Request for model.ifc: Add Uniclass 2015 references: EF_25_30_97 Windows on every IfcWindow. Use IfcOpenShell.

First a look at what the model holds.

```python
import ifcopenshell

model = ifcopenshell.open("model.ifc")
print(model.schema)
print("classifications:", [c.Name for c in model.by_type("IfcClassification")])
for ifc_class in ("IfcDoor", "IfcRoof", "IfcStair", "IfcWall", "IfcWindow"):
    print(ifc_class, len(model.by_type(ifc_class)))
```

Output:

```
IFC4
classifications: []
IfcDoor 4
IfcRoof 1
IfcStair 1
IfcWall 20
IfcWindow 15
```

```python
import ifcopenshell
import ifcopenshell.api.classification

model = ifcopenshell.open("model.ifc")

system = ifcopenshell.api.classification.add_classification(model, classification="Uniclass 2015")

codes = {
    "IfcWindow": ("EF_25_30_97", "Windows"),
}
for ifc_class, (code, name) in codes.items():
    products = model.by_type(ifc_class)
    ifcopenshell.api.classification.add_reference(
        model, products=products, classification=system, identification=code, name=name
    )
    print(code, len(products))

model.write("model_updated.ifc")
```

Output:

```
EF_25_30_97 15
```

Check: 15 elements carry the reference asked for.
